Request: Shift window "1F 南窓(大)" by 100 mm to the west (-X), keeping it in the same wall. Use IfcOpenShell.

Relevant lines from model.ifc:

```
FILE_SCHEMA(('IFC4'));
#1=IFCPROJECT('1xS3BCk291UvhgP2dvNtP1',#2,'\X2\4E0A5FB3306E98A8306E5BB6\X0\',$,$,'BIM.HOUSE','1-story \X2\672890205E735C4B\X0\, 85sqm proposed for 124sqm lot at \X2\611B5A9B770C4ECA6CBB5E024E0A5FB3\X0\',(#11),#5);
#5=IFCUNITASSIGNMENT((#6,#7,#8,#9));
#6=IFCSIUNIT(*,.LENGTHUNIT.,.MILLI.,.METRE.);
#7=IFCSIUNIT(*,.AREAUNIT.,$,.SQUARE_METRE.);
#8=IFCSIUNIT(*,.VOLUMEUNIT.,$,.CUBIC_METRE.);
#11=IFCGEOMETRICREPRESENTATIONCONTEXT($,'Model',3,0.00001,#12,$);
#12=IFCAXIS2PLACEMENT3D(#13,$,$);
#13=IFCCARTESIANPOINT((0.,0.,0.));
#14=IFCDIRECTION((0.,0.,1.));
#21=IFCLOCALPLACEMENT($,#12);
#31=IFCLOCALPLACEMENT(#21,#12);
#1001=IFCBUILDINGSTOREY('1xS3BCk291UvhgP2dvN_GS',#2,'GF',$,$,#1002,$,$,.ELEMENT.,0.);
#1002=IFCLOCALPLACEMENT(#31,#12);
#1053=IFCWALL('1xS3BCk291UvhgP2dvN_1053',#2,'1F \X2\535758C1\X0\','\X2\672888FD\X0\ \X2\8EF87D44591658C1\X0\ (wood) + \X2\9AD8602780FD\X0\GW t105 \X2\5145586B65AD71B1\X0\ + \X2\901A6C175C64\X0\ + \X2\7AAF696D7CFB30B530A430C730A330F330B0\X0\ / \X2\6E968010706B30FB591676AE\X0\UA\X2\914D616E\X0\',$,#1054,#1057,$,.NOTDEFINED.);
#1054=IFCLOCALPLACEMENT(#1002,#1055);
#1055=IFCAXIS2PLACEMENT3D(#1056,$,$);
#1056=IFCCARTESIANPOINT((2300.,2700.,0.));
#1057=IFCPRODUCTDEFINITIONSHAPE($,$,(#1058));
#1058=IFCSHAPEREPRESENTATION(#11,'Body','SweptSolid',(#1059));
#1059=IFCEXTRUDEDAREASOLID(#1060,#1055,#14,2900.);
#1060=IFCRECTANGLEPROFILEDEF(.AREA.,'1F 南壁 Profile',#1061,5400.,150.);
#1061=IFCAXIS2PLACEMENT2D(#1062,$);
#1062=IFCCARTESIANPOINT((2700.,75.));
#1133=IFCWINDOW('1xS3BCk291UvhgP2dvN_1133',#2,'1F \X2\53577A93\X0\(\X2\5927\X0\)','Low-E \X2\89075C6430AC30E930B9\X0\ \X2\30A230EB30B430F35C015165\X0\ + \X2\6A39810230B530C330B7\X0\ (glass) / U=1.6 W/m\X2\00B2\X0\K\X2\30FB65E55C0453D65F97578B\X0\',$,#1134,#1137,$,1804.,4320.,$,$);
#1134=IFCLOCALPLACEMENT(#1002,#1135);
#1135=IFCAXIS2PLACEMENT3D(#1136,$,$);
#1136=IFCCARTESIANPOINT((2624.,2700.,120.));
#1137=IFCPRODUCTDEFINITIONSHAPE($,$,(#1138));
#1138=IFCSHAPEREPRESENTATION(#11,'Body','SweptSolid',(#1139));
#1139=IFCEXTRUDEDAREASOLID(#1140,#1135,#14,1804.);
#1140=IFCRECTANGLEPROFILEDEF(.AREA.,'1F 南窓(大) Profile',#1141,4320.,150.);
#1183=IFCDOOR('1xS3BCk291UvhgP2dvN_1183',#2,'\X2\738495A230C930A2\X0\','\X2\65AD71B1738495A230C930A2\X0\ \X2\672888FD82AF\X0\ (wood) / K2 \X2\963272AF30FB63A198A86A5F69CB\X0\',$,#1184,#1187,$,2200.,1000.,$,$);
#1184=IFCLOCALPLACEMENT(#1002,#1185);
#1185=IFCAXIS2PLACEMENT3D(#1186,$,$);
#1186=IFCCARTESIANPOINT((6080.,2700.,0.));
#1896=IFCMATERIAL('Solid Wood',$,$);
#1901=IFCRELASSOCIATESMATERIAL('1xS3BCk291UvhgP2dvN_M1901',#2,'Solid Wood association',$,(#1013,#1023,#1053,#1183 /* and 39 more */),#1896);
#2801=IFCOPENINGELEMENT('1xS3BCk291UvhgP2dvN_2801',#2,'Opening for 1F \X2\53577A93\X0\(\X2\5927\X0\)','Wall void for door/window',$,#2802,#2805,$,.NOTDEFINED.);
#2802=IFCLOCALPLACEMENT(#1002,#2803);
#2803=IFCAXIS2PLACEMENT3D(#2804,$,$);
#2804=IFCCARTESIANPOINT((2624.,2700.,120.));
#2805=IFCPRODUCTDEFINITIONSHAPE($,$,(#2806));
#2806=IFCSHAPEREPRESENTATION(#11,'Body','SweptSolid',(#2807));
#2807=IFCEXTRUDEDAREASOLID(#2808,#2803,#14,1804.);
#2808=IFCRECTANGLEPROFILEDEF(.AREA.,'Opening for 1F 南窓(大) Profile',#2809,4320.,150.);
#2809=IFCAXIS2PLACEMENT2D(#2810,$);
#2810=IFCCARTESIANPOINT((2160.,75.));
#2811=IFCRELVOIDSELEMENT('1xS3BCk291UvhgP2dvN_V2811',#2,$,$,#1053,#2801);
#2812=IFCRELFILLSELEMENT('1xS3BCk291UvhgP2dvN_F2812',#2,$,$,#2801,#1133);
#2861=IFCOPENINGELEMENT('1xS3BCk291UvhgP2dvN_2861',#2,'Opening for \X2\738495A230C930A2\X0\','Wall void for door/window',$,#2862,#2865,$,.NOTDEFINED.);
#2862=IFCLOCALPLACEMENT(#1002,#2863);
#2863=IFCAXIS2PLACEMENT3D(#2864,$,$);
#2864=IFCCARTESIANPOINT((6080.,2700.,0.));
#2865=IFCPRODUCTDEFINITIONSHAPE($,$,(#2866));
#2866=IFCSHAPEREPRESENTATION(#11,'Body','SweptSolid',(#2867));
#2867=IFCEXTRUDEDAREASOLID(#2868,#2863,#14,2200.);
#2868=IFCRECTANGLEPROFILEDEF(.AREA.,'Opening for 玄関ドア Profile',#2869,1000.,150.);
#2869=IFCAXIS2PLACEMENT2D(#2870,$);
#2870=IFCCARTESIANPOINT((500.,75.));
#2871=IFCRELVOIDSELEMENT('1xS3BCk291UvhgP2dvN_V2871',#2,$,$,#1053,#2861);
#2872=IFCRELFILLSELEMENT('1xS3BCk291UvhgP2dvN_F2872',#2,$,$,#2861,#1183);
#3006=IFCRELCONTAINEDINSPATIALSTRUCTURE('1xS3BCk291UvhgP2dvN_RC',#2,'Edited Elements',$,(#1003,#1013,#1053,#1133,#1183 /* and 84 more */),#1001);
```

```python
import ifcopenshell
import ifcopenshell.api.geometry
import ifcopenshell.util.placement
import ifcopenshell.util.unit

model = ifcopenshell.open("model.ifc")
unit_scale = ifcopenshell.util.unit.calculate_unit_scale(model)

window = model.by_guid("1xS3BCk291UvhgP2dvN_1133")
opening = window.FillsVoids[0].RelatingOpeningElement
wall = opening.VoidsElements[0].RelatingBuildingElement

wall_matrix = ifcopenshell.util.placement.get_local_placement(wall.ObjectPlacement)
shift = wall_matrix[:3, 0] * -0.1 / unit_scale
before = ifcopenshell.util.placement.get_local_placement(window.ObjectPlacement)[:3, 3].copy()

# The window is not placed relative to its opening, so move both.
for product in (opening, window):
    matrix = ifcopenshell.util.placement.get_local_placement(product.ObjectPlacement)
    matrix[:3, 3] += shift
    ifcopenshell.api.geometry.edit_object_placement(model, product=product, matrix=matrix, is_si=False)

after = ifcopenshell.util.placement.get_local_placement(window.ObjectPlacement)[:3, 3]
print("window moved by", (after - before).round(3) + 0.0)

model.write("model_updated.ifc")
```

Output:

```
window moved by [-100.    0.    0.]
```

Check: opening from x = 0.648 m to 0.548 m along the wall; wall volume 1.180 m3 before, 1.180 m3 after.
